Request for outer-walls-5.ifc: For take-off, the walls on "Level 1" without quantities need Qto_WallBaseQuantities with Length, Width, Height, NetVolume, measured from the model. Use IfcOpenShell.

First a look at what the model holds.

```python
import ifcopenshell
import ifcopenshell.util.element
import ifcopenshell.util.unit

model = ifcopenshell.open("outer-walls-5.ifc")
print(model.schema)
for unit_type in ("LENGTHUNIT", "AREAUNIT", "VOLUMEUNIT"):
    print(unit_type, ifcopenshell.util.unit.calculate_unit_scale(model, unit_type))
storey = next(s for s in model.by_type("IfcBuildingStorey") if s.Name == "Level 1")
walls = [e for e in ifcopenshell.util.element.get_decomposition(storey) if e.is_a("IfcWall")]
for e in sorted(walls, key=lambda e: e.id()):
    print(e.id(), e.is_a(), e.Name, list(ifcopenshell.util.element.get_psets(e, qtos_only=True)), sep=" | ")
```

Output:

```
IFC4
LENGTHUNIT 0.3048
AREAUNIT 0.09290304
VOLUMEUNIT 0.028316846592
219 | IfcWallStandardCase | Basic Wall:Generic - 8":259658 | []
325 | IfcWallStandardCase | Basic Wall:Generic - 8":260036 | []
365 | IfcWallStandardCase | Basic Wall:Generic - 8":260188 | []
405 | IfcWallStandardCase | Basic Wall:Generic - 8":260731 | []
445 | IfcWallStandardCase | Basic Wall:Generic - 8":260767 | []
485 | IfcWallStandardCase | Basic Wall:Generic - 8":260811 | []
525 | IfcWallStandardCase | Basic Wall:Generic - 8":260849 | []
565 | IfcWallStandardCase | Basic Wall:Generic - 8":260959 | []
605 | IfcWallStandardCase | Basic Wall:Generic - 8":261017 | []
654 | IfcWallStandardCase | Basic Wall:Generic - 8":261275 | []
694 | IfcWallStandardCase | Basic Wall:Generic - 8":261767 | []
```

```python
import ifcopenshell
import ifcopenshell.api.pset
import ifcopenshell.geom
import ifcopenshell.util.element
import ifcopenshell.util.shape
import ifcopenshell.util.unit

model = ifcopenshell.open("outer-walls-5.ifc")
unit_scale = ifcopenshell.util.unit.calculate_unit_scale(model)
volume_scale = ifcopenshell.util.unit.calculate_unit_scale(model, "VOLUMEUNIT")
settings = ifcopenshell.geom.settings()

storey = next(s for s in model.by_type("IfcBuildingStorey") if s.Name == "Level 1")
walls = [e for e in ifcopenshell.util.element.get_decomposition(storey) if e.is_a("IfcWall")]

for e in sorted(walls, key=lambda e: e.id()):
    if ifcopenshell.util.element.get_psets(e, qtos_only=True, should_inherit=False):
        continue
    # Geometry comes back in metres, in the element's own axes.
    shape = ifcopenshell.geom.create_shape(settings, e)
    values = {
        "Length": ifcopenshell.util.shape.get_x(shape.geometry) / unit_scale,
        "Width": ifcopenshell.util.shape.get_y(shape.geometry) / unit_scale,
        "Height": ifcopenshell.util.shape.get_z(shape.geometry) / unit_scale,
        "NetVolume": ifcopenshell.util.shape.get_volume(shape.geometry) / volume_scale,
    }
    qto = ifcopenshell.api.pset.add_qto(model, product=e, name="Qto_WallBaseQuantities")
    ifcopenshell.api.pset.edit_qto(model, qto=qto, properties=values)
    print(e.id(), {k: round(v, 3) for k, v in values.items()})

model.write("outer-walls-5_updated.ifc")
```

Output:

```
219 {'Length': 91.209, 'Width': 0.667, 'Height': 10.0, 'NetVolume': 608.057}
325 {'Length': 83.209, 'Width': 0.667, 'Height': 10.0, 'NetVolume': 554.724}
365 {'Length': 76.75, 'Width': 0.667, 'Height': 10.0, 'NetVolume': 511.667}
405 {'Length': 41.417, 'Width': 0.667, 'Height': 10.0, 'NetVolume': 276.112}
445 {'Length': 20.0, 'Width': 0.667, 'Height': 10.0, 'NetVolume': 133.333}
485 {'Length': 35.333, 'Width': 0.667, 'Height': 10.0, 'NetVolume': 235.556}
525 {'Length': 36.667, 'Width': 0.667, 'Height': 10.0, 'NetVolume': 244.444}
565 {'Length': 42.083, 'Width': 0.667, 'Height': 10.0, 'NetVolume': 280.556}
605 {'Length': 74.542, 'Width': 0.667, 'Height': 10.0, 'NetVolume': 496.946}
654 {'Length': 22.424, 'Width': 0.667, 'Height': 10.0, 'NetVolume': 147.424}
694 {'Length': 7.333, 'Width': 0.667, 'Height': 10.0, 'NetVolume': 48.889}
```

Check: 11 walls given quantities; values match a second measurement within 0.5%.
